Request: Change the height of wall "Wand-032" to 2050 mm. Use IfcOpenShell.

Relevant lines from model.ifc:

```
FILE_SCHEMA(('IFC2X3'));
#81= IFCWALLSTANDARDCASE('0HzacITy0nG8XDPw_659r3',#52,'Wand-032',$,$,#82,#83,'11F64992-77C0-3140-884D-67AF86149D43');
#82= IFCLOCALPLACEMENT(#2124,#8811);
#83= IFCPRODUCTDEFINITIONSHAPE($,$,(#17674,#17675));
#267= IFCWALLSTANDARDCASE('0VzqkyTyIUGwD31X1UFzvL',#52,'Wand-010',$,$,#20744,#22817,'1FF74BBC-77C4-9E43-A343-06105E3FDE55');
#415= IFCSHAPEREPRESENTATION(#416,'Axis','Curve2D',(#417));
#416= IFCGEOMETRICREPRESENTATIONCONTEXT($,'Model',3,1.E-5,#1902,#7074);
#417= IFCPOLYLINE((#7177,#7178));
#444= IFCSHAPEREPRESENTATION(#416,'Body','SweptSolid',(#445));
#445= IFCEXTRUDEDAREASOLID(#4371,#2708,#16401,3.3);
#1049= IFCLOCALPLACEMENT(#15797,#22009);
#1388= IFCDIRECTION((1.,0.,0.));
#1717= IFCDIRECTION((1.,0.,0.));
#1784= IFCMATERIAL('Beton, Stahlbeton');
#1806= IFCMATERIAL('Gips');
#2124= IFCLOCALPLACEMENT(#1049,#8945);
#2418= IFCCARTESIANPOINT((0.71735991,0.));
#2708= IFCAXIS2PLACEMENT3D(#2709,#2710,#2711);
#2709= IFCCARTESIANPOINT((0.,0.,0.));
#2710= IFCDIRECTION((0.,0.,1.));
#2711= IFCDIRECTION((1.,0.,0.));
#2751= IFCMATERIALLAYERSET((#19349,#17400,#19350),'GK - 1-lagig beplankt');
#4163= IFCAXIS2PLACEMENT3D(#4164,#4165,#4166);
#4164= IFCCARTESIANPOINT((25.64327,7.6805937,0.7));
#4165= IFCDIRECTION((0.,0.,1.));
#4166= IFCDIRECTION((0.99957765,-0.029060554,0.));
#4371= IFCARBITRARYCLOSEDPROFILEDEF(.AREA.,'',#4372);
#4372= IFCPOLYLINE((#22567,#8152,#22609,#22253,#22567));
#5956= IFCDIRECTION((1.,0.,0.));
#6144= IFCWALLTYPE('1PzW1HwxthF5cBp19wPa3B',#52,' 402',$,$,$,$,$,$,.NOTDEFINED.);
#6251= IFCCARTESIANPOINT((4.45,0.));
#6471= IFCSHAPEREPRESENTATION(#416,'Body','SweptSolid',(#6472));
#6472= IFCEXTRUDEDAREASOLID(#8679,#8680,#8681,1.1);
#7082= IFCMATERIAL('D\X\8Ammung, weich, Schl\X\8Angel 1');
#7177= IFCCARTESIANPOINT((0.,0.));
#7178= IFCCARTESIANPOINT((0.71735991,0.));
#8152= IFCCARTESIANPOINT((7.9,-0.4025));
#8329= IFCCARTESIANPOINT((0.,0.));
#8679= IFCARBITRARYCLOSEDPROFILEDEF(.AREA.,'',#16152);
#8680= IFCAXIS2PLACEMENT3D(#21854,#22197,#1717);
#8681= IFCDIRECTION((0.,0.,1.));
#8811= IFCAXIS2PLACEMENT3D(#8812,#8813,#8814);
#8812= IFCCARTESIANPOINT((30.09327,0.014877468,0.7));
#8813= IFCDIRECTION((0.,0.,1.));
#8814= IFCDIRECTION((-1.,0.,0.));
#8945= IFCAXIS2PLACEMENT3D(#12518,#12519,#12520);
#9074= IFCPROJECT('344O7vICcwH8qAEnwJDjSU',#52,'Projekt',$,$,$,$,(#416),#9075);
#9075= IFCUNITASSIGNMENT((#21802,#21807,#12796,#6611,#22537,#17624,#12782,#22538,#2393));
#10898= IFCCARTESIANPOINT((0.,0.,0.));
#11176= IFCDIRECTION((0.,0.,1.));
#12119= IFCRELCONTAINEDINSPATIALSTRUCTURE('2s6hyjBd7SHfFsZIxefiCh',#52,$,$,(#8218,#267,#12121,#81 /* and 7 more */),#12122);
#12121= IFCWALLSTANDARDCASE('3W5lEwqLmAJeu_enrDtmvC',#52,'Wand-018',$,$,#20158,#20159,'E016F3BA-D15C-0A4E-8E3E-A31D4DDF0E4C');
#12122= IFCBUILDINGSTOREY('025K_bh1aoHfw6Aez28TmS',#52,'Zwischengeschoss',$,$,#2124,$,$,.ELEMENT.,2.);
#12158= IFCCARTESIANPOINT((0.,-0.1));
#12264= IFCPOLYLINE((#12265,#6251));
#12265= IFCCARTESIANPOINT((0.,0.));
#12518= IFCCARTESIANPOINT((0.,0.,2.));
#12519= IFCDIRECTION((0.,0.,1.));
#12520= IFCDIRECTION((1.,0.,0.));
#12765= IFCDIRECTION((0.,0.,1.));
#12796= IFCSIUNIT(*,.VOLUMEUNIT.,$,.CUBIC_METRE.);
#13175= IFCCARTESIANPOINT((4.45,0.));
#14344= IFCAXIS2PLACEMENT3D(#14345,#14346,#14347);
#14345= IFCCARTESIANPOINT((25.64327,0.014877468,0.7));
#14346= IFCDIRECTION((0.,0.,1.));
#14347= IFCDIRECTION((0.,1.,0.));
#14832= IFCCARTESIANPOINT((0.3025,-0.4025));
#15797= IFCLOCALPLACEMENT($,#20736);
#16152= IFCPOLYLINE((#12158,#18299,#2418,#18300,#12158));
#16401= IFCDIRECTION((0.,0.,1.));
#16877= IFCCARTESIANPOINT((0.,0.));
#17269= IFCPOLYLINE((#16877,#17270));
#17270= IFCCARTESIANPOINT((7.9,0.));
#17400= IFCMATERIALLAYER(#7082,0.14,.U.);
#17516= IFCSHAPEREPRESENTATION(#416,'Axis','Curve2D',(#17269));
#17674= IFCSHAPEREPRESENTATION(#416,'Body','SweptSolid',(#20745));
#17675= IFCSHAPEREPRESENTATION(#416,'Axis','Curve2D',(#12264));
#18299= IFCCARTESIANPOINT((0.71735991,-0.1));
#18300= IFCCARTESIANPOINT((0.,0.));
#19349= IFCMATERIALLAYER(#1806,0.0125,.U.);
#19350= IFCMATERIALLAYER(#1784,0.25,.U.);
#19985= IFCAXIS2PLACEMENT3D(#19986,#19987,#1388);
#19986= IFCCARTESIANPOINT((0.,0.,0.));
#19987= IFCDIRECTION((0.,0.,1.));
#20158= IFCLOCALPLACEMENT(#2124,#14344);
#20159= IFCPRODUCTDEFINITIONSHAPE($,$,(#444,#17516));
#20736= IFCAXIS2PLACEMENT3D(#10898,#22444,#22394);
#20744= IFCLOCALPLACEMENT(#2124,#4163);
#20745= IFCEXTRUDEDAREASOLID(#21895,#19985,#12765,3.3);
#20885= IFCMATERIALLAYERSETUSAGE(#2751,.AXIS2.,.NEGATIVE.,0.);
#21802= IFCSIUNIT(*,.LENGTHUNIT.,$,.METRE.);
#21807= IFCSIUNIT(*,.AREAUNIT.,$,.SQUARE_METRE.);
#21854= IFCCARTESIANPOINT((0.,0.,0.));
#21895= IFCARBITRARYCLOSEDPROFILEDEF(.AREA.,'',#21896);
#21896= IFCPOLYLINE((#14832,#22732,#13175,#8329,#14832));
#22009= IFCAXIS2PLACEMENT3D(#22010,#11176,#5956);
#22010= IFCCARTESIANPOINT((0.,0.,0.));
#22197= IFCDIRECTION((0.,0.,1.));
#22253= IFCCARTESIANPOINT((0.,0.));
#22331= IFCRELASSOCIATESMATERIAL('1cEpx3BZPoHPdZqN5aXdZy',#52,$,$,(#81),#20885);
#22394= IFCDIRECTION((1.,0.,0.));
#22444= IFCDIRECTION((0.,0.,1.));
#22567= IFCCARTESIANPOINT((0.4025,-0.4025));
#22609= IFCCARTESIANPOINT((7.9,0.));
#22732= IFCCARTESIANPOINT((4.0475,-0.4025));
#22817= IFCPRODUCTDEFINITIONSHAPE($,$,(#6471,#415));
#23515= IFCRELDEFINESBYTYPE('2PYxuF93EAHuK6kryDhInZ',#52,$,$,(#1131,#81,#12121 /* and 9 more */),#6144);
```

```python
import ifcopenshell
import ifcopenshell.geom
import ifcopenshell.util.shape

model = ifcopenshell.open("model.ifc")
settings = ifcopenshell.geom.settings()


def volume(element):
    """Net volume in cubic metres, openings subtracted."""
    shape = ifcopenshell.geom.create_shape(settings, element)
    return ifcopenshell.util.shape.get_volume(shape.geometry)


wall = model.by_guid("0HzacITy0nG8XDPw_659r3")
before = volume(wall)

body = next(r for r in wall.Representation.Representations if r.RepresentationIdentifier == "Body")
solid = body.Items[0]
old_height = solid.Depth
solid.Depth = 2.05
after = volume(wall)

print(f"height {old_height:g} -> {solid.Depth:g}, volume {before:.3f} -> {after:.3f} m3")

model.write("model_updated.ifc")
```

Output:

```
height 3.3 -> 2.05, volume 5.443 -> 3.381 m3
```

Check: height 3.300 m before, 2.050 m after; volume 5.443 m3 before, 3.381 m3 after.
